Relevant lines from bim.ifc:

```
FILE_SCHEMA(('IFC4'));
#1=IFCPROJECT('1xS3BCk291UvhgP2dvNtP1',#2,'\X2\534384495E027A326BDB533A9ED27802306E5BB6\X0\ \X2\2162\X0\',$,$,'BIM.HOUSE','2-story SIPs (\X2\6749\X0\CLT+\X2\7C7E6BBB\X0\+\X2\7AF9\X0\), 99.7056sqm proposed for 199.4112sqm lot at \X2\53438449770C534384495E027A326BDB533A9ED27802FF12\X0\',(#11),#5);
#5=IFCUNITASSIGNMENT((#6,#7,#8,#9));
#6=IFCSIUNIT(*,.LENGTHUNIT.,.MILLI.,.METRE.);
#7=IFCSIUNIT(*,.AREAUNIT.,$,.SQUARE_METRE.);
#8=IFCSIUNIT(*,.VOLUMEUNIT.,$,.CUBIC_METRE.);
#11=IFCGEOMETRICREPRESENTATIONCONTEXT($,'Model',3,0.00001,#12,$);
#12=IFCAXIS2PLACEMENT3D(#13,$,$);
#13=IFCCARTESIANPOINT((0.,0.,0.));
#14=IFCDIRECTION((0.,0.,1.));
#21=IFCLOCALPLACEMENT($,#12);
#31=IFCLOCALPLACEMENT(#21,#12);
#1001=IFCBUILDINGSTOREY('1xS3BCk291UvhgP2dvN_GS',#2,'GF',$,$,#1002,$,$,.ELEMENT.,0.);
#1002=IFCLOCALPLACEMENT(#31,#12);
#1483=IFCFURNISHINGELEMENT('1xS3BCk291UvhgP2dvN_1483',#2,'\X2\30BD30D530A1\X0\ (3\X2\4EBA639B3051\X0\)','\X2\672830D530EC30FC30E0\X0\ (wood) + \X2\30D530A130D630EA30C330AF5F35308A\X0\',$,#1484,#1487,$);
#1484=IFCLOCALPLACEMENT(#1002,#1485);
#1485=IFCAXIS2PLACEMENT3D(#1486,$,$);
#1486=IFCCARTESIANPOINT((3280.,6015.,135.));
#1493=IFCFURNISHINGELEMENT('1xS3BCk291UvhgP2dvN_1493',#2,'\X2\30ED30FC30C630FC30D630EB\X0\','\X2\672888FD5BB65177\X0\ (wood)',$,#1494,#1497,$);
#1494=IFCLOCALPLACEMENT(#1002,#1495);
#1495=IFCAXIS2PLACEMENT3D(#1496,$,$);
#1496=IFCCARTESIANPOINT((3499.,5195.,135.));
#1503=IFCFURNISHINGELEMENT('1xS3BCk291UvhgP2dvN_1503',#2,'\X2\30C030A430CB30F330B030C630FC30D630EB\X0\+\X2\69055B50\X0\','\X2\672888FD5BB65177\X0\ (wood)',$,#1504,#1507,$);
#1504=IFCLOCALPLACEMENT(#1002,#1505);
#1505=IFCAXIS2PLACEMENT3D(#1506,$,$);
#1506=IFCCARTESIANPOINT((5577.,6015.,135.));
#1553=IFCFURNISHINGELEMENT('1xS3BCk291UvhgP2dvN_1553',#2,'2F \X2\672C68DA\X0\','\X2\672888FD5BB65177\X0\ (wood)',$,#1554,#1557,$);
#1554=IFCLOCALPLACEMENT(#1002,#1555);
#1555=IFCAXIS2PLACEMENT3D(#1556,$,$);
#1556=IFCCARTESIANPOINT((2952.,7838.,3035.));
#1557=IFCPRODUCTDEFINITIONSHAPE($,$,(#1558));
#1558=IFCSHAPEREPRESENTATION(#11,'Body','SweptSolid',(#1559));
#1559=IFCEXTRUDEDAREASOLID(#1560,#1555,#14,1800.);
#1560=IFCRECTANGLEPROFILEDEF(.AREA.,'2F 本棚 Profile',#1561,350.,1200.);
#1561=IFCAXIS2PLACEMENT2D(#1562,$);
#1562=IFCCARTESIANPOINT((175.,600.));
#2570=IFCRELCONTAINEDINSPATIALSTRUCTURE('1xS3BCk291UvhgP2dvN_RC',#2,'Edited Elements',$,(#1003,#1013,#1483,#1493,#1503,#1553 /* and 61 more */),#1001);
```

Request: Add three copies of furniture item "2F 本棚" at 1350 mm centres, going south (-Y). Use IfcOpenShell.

```python
import numpy as np
import ifcopenshell
import ifcopenshell.api.geometry
import ifcopenshell.api.root
import ifcopenshell.util.element
import ifcopenshell.util.placement

model = ifcopenshell.open("bim.ifc")


def reuse_history(source, copy):
    """copy_class also copies each property set's owner history, people and application; keep the originals."""
    for rel in copy.IsDefinedBy:
        if rel.is_a("IfcRelDefinesByProperties") and (history := rel.RelatingPropertyDefinition.OwnerHistory):
            rel.RelatingPropertyDefinition.OwnerHistory = source.OwnerHistory
            ifcopenshell.util.element.remove_deep2(model, history)


source = model.by_guid("1xS3BCk291UvhgP2dvN_1553")
base = ifcopenshell.util.placement.get_local_placement(source.ObjectPlacement)
step = np.array([0.0, -1.0, 0.0]) * 1350.0

for i in range(1, 4):
    copy = ifcopenshell.api.root.copy_class(model, product=source)
    copy.Representation = ifcopenshell.util.element.copy_deep(
        model, source.Representation, exclude=["IfcGeometricRepresentationContext", "IfcRepresentationMap"]
    )
    reuse_history(source, copy)
    matrix = base.copy()
    matrix[:3, 3] += i * step
    print("added at", matrix[:3, 3].round(3) + 0.0)
    ifcopenshell.api.geometry.edit_object_placement(model, product=copy, matrix=matrix, is_si=False)

model.write("bim_edited.ifc")
```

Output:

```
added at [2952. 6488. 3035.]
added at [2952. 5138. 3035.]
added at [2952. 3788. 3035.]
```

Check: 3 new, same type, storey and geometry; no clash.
